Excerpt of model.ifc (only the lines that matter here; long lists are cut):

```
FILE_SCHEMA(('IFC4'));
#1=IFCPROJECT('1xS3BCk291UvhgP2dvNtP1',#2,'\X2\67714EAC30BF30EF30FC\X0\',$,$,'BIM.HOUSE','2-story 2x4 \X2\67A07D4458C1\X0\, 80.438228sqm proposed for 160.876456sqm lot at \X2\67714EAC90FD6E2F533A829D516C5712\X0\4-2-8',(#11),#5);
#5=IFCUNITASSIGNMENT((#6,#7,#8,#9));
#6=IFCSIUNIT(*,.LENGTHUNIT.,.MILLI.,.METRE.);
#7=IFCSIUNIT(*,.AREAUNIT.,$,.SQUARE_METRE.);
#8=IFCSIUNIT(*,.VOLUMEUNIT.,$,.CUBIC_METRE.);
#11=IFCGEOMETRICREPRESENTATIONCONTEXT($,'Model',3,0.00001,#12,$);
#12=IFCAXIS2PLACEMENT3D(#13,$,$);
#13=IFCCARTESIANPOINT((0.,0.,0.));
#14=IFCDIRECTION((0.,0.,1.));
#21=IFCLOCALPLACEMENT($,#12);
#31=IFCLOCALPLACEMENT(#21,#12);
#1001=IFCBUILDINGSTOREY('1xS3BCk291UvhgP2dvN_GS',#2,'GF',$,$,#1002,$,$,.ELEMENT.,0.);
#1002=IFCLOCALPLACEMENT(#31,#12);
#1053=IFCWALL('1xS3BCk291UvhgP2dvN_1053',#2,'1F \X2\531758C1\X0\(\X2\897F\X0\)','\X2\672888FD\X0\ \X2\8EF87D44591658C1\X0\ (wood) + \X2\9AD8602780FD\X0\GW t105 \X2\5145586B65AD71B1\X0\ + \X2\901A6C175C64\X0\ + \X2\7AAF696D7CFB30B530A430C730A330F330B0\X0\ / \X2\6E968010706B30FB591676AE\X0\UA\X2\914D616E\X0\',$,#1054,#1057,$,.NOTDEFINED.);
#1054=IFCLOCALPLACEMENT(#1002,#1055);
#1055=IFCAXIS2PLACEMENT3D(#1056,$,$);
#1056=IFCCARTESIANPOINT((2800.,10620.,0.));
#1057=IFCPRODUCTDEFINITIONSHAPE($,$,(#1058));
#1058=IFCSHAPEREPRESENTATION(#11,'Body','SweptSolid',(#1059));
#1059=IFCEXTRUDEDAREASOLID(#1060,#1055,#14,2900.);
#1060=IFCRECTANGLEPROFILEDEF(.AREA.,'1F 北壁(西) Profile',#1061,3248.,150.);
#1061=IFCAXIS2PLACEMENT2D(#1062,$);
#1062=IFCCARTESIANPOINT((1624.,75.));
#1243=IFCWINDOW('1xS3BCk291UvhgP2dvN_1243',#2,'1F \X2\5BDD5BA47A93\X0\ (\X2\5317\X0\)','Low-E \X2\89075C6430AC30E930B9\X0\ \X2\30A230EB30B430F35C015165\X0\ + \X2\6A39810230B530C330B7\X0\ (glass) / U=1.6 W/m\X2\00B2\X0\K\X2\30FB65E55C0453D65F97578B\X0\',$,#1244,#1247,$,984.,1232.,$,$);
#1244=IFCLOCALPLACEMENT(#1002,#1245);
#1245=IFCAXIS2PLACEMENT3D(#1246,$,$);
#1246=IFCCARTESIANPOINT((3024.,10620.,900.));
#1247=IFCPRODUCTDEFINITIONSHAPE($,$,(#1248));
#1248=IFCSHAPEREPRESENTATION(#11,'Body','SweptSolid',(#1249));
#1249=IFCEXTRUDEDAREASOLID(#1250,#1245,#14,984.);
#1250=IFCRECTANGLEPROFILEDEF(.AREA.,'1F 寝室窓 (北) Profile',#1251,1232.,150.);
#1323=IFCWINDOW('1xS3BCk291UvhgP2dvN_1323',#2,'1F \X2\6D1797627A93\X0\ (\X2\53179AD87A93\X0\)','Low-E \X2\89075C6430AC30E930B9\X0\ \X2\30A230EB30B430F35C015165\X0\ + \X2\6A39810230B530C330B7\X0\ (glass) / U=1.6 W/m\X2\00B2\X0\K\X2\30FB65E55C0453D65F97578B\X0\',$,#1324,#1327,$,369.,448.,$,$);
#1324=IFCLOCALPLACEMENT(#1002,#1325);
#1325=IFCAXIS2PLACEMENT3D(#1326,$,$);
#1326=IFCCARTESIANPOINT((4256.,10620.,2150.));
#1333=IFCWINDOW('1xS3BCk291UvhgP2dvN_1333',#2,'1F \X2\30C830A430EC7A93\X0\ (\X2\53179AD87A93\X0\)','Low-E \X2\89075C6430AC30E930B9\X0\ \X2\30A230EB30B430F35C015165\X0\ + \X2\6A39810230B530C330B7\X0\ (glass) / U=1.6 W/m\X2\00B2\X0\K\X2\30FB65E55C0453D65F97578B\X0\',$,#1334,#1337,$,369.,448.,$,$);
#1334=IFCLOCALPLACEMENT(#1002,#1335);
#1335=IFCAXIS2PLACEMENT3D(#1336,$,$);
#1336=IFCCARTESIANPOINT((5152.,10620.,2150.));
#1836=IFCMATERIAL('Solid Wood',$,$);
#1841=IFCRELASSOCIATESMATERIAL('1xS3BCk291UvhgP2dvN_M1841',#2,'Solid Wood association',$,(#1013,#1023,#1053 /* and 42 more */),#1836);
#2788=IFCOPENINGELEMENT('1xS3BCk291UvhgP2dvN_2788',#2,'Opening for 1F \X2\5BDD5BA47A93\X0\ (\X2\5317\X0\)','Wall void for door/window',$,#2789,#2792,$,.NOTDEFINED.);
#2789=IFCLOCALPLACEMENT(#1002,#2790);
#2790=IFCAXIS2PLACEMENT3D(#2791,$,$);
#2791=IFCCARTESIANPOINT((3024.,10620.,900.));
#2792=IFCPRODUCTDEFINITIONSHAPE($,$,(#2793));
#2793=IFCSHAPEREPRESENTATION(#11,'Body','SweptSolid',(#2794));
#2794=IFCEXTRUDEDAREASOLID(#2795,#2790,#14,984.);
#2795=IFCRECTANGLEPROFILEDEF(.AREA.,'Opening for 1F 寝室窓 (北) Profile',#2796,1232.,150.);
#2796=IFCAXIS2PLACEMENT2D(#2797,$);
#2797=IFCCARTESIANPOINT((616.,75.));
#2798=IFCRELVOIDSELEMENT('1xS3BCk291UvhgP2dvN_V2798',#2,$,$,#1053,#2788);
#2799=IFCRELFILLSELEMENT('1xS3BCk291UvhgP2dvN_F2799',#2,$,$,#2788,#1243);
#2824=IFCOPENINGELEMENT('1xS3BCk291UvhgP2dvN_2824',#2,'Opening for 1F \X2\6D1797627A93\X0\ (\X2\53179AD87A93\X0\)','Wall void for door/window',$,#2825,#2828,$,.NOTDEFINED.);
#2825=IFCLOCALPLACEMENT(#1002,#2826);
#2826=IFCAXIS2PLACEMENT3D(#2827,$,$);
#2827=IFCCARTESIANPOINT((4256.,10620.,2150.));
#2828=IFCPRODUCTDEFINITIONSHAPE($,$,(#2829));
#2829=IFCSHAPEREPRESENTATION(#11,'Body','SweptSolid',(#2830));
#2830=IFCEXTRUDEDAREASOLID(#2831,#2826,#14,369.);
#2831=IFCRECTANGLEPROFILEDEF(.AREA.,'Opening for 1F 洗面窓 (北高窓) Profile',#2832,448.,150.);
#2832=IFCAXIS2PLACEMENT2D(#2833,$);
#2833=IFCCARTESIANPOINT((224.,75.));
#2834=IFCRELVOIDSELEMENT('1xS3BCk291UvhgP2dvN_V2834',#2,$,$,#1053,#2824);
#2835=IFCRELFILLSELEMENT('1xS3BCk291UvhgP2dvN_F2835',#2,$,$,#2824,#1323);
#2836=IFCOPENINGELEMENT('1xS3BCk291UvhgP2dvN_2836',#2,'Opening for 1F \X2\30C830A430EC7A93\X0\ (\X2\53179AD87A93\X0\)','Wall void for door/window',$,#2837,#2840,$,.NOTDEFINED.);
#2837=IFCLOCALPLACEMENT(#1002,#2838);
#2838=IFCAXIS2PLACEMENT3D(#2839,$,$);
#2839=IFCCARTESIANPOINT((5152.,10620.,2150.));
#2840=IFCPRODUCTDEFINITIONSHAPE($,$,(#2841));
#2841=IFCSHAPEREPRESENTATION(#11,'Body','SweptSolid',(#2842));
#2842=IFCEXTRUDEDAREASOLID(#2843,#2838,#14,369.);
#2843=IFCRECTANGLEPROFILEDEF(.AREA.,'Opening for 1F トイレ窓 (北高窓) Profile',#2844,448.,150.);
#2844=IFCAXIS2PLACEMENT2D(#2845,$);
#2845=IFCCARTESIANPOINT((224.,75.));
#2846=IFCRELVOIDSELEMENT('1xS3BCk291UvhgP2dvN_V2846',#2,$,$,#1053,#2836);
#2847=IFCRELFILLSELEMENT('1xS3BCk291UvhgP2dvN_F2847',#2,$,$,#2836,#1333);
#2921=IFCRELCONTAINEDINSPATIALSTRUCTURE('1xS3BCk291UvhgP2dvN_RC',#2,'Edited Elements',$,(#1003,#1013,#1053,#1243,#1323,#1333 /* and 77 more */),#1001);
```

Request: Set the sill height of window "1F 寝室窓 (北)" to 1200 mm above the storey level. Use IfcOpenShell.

```python
import numpy as np
import ifcopenshell
import ifcopenshell.api.geometry
import ifcopenshell.geom
import ifcopenshell.util.element
import ifcopenshell.util.placement
import ifcopenshell.util.shape
import ifcopenshell.util.unit

model = ifcopenshell.open("model.ifc")
unit_scale = ifcopenshell.util.unit.calculate_unit_scale(model)

window = model.by_guid("1xS3BCk291UvhgP2dvN_1243")
opening = window.FillsVoids[0].RelatingOpeningElement
storey = ifcopenshell.util.element.get_container(window, ifc_class="IfcBuildingStorey")
level = ifcopenshell.util.placement.get_local_placement(storey.ObjectPlacement)[2, 3]

# The opening's origin need not be at the sill, so measure its lowest point.
shape = ifcopenshell.geom.create_shape(ifcopenshell.geom.settings(), opening)
bottom = ifcopenshell.util.shape.get_shape_bottom_elevation(shape, shape.geometry) / unit_scale
dz = level + 1200.0 - bottom

shift = np.array([0.0, 0.0, dz])
# The window is not placed relative to its opening, so move both.
for product in (opening, window):
    matrix = ifcopenshell.util.placement.get_local_placement(product.ObjectPlacement)
    matrix[:3, 3] += shift
    ifcopenshell.api.geometry.edit_object_placement(model, product=product, matrix=matrix, is_si=False)

print(f"moved by {dz * unit_scale:+.3f} m")

model.write("model-out.ifc")
```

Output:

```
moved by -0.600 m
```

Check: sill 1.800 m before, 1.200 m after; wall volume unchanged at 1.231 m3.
